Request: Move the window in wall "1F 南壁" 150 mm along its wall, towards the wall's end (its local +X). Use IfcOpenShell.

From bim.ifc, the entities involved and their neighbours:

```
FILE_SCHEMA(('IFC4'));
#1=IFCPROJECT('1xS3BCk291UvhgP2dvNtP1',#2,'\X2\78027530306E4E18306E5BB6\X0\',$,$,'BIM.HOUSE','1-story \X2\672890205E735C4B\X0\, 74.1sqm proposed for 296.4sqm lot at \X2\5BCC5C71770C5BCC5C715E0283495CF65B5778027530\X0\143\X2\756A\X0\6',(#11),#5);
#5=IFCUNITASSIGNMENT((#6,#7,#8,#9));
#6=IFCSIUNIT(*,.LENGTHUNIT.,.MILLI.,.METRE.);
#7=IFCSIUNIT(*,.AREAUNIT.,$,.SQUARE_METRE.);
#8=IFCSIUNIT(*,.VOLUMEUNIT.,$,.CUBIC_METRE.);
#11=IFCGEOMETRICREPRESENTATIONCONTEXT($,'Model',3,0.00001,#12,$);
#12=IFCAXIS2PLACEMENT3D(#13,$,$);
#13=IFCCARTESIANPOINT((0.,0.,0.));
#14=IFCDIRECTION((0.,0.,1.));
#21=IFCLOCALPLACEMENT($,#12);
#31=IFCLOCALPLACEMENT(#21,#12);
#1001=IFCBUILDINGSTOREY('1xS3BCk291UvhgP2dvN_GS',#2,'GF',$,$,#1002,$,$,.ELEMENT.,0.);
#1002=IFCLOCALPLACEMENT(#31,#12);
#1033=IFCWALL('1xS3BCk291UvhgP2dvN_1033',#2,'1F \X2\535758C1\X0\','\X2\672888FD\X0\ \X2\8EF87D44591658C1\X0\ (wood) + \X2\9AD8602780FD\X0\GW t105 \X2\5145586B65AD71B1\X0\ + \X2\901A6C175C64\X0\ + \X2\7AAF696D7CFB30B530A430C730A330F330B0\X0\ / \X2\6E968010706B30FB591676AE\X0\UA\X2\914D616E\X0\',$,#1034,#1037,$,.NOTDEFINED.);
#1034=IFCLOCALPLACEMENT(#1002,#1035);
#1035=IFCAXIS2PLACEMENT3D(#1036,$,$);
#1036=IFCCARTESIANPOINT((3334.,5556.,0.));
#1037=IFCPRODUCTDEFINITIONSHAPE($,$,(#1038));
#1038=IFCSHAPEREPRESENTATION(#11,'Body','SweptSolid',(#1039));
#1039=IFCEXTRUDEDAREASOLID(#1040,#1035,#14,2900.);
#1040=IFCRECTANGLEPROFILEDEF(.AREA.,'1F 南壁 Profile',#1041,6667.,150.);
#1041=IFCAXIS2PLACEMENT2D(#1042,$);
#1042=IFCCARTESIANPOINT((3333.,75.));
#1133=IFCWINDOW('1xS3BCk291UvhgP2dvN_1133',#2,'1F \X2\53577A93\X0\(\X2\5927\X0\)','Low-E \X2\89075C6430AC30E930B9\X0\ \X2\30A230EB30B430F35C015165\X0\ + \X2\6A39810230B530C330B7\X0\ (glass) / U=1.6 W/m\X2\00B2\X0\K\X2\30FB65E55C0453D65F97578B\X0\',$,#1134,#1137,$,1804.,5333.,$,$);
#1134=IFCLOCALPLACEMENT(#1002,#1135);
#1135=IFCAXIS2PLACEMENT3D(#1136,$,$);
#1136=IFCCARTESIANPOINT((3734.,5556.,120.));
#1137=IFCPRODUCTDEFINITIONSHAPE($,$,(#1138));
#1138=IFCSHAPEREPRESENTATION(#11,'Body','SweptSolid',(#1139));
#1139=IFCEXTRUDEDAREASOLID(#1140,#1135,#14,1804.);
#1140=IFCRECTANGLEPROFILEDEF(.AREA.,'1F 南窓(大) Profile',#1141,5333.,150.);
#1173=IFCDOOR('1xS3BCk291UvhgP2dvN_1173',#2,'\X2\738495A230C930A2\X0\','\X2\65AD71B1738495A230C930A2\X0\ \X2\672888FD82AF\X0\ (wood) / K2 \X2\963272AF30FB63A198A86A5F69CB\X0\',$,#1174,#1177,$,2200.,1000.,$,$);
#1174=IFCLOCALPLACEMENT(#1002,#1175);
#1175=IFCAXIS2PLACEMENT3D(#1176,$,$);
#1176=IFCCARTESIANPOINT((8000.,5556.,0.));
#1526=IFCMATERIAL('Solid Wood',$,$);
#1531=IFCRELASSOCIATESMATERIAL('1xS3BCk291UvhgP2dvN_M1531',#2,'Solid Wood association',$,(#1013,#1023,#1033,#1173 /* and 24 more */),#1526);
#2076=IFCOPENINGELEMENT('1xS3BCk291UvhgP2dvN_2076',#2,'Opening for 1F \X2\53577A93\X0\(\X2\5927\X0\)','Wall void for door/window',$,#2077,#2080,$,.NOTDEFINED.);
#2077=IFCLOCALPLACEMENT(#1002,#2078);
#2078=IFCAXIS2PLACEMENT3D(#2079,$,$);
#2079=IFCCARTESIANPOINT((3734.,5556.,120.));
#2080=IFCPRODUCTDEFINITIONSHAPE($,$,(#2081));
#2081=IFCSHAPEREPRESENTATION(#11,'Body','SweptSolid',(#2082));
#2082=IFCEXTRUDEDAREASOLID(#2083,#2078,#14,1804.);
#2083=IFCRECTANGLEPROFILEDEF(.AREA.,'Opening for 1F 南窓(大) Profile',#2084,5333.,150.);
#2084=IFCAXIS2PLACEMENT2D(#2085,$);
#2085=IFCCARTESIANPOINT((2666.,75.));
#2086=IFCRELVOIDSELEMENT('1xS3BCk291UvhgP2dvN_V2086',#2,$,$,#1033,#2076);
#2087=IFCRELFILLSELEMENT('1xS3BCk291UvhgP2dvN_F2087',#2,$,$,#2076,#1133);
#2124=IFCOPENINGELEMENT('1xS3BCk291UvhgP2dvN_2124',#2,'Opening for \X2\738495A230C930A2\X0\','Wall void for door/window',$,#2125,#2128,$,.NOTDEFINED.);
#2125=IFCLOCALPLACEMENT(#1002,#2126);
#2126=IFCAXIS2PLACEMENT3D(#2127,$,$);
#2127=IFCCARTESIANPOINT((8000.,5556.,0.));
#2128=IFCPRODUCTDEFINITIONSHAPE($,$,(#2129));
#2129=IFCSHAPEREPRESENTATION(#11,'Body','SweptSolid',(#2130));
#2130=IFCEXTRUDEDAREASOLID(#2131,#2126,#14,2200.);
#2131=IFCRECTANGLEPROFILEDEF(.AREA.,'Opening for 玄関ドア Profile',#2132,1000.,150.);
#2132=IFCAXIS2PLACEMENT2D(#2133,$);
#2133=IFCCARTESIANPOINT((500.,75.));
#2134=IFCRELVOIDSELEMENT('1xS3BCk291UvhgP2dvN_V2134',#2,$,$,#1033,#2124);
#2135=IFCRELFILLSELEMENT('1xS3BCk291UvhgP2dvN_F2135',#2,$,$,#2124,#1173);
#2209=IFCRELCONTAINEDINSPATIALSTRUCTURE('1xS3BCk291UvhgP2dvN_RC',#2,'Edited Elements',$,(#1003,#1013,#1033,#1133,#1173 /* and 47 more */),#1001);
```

```python
import ifcopenshell
import ifcopenshell.api.geometry
import ifcopenshell.util.placement

model = ifcopenshell.open("bim.ifc")

window = model.by_id(1133)
opening = window.FillsVoids[0].RelatingOpeningElement
wall = opening.VoidsElements[0].RelatingBuildingElement

wall_matrix = ifcopenshell.util.placement.get_local_placement(wall.ObjectPlacement)
shift = wall_matrix[:3, 0] * 150.0
before = ifcopenshell.util.placement.get_local_placement(window.ObjectPlacement)[:3, 3].copy()

# The window is not placed relative to its opening, so move both.
for product in (opening, window):
    matrix = ifcopenshell.util.placement.get_local_placement(product.ObjectPlacement)
    matrix[:3, 3] += shift
    ifcopenshell.api.geometry.edit_object_placement(model, product=product, matrix=matrix, is_si=False)

after = ifcopenshell.util.placement.get_local_placement(window.ObjectPlacement)[:3, 3]
print("window moved by", (after - before).round(3) + 0.0)

model.write("bim_edited.ifc")
```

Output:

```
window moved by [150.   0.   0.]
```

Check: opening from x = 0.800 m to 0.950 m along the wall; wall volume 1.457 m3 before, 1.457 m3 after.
